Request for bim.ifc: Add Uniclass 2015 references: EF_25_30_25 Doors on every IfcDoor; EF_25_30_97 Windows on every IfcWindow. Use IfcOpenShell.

First a look at what the model holds.

```python
import ifcopenshell

model = ifcopenshell.open("bim.ifc")
print(model.schema)
print("classifications:", [c.Name for c in model.by_type("IfcClassification")])
for ifc_class in ("IfcDoor", "IfcRoof", "IfcStair", "IfcWall", "IfcWindow"):
    print(ifc_class, len(model.by_type(ifc_class)))
```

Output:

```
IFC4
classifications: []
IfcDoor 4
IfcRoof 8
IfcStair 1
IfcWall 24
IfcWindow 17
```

```python
import ifcopenshell
import ifcopenshell.api.classification

model = ifcopenshell.open("bim.ifc")

system = ifcopenshell.api.classification.add_classification(model, classification="Uniclass 2015")

codes = {
    "IfcDoor": ("EF_25_30_25", "Doors"),
    "IfcWindow": ("EF_25_30_97", "Windows"),
}
for ifc_class, (code, name) in codes.items():
    products = model.by_type(ifc_class)
    ifcopenshell.api.classification.add_reference(
        model, products=products, classification=system, identification=code, name=name
    )
    print(code, len(products))

model.write("bim-out.ifc")
```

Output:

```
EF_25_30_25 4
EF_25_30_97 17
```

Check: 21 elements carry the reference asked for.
